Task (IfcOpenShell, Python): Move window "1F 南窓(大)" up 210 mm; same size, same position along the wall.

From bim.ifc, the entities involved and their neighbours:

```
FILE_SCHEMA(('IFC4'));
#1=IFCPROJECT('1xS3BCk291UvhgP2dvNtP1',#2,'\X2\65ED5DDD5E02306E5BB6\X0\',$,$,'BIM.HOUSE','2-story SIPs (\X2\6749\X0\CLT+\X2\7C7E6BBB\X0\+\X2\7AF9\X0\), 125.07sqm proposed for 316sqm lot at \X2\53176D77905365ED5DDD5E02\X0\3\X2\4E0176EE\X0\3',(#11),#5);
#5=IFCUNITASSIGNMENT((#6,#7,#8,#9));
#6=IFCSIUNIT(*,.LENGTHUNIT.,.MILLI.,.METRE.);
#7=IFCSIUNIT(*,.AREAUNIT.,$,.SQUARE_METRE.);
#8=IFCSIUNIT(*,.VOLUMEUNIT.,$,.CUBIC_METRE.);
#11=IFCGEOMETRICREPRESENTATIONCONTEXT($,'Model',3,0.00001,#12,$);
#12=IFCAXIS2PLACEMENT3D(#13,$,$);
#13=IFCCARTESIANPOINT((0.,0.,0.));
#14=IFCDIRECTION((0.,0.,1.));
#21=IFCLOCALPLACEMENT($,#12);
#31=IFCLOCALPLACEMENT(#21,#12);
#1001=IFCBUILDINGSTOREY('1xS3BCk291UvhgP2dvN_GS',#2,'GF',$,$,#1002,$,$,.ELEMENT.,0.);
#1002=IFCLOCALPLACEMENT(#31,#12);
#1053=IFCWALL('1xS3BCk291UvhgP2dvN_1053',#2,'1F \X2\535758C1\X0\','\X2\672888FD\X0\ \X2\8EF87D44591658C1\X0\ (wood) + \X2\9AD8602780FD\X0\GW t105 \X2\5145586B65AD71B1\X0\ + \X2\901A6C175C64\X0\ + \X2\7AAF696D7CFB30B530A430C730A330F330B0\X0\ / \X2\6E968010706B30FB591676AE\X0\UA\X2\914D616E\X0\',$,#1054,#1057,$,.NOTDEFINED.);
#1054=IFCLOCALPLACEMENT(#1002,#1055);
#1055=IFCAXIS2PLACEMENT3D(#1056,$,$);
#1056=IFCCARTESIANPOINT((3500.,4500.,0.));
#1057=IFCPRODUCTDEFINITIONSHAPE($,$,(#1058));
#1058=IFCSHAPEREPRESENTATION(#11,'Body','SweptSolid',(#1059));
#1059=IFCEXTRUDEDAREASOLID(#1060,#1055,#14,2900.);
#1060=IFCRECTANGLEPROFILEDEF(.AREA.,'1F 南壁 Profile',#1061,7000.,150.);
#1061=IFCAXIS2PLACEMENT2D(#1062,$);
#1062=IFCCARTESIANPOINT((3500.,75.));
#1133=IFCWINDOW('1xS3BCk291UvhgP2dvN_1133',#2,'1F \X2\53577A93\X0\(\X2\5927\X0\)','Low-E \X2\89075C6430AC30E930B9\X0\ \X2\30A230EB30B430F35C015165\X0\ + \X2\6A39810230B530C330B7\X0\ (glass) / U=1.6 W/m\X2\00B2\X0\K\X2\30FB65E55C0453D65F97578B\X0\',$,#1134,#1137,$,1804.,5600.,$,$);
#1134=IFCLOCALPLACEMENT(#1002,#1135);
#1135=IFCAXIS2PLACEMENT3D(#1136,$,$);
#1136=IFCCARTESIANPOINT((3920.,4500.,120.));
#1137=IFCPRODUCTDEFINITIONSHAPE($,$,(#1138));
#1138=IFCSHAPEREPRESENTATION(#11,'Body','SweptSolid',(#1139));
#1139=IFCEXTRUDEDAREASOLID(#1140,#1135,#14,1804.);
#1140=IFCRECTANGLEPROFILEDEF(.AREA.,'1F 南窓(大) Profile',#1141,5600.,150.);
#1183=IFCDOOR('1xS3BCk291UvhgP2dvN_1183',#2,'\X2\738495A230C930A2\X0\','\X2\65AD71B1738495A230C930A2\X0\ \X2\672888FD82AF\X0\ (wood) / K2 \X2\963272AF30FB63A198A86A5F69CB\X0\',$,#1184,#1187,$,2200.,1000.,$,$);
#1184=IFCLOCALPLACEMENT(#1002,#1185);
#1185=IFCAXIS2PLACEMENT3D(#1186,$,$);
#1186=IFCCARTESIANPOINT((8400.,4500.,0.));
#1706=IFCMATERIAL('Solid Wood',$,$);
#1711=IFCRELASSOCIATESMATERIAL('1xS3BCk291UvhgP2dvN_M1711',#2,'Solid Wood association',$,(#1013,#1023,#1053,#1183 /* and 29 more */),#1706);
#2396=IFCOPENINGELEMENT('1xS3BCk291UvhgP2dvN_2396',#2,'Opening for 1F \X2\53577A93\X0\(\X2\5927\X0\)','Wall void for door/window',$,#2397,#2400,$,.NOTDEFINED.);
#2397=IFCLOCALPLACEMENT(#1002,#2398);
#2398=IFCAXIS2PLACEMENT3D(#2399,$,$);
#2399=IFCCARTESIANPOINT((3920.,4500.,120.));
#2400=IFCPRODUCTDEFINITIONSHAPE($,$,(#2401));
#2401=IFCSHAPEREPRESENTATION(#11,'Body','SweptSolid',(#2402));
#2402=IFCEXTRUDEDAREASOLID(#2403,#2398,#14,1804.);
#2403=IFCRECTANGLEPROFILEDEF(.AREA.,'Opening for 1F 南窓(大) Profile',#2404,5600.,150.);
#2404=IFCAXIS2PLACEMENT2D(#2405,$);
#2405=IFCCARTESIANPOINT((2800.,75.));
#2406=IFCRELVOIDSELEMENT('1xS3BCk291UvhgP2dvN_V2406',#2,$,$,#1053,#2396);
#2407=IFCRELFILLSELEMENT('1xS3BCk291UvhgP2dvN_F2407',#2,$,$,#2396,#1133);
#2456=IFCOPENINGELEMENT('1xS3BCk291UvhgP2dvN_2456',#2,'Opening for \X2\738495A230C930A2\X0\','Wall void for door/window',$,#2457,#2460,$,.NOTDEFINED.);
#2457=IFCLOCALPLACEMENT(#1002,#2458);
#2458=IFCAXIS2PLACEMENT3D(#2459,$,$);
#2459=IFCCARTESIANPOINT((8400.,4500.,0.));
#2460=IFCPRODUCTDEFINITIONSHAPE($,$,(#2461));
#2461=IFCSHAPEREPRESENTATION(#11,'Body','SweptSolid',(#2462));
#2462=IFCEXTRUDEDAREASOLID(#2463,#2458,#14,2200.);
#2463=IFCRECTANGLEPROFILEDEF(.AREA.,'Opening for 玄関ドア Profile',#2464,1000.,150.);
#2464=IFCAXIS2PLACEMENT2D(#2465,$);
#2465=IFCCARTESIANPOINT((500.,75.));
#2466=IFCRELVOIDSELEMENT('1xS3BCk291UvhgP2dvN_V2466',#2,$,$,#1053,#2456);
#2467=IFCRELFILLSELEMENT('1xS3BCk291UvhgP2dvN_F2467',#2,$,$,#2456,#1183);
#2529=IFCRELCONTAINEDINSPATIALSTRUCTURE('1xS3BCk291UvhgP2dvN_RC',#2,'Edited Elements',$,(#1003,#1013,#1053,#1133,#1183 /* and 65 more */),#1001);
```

```python
import numpy as np
import ifcopenshell
import ifcopenshell.api.geometry
import ifcopenshell.util.placement
import ifcopenshell.util.unit

model = ifcopenshell.open("bim.ifc")
unit_scale = ifcopenshell.util.unit.calculate_unit_scale(model)

window = model.by_guid("1xS3BCk291UvhgP2dvN_1133")
opening = window.FillsVoids[0].RelatingOpeningElement
dz = 0.21 / unit_scale

shift = np.array([0.0, 0.0, dz])
# The window is not placed relative to its opening, so move both.
for product in (opening, window):
    matrix = ifcopenshell.util.placement.get_local_placement(product.ObjectPlacement)
    matrix[:3, 3] += shift
    ifcopenshell.api.geometry.edit_object_placement(model, product=product, matrix=matrix, is_si=False)

print(f"moved by {dz * unit_scale:+.3f} m")

model.write("bim_v2.ifc")
```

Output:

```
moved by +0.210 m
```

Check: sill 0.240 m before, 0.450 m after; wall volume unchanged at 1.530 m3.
